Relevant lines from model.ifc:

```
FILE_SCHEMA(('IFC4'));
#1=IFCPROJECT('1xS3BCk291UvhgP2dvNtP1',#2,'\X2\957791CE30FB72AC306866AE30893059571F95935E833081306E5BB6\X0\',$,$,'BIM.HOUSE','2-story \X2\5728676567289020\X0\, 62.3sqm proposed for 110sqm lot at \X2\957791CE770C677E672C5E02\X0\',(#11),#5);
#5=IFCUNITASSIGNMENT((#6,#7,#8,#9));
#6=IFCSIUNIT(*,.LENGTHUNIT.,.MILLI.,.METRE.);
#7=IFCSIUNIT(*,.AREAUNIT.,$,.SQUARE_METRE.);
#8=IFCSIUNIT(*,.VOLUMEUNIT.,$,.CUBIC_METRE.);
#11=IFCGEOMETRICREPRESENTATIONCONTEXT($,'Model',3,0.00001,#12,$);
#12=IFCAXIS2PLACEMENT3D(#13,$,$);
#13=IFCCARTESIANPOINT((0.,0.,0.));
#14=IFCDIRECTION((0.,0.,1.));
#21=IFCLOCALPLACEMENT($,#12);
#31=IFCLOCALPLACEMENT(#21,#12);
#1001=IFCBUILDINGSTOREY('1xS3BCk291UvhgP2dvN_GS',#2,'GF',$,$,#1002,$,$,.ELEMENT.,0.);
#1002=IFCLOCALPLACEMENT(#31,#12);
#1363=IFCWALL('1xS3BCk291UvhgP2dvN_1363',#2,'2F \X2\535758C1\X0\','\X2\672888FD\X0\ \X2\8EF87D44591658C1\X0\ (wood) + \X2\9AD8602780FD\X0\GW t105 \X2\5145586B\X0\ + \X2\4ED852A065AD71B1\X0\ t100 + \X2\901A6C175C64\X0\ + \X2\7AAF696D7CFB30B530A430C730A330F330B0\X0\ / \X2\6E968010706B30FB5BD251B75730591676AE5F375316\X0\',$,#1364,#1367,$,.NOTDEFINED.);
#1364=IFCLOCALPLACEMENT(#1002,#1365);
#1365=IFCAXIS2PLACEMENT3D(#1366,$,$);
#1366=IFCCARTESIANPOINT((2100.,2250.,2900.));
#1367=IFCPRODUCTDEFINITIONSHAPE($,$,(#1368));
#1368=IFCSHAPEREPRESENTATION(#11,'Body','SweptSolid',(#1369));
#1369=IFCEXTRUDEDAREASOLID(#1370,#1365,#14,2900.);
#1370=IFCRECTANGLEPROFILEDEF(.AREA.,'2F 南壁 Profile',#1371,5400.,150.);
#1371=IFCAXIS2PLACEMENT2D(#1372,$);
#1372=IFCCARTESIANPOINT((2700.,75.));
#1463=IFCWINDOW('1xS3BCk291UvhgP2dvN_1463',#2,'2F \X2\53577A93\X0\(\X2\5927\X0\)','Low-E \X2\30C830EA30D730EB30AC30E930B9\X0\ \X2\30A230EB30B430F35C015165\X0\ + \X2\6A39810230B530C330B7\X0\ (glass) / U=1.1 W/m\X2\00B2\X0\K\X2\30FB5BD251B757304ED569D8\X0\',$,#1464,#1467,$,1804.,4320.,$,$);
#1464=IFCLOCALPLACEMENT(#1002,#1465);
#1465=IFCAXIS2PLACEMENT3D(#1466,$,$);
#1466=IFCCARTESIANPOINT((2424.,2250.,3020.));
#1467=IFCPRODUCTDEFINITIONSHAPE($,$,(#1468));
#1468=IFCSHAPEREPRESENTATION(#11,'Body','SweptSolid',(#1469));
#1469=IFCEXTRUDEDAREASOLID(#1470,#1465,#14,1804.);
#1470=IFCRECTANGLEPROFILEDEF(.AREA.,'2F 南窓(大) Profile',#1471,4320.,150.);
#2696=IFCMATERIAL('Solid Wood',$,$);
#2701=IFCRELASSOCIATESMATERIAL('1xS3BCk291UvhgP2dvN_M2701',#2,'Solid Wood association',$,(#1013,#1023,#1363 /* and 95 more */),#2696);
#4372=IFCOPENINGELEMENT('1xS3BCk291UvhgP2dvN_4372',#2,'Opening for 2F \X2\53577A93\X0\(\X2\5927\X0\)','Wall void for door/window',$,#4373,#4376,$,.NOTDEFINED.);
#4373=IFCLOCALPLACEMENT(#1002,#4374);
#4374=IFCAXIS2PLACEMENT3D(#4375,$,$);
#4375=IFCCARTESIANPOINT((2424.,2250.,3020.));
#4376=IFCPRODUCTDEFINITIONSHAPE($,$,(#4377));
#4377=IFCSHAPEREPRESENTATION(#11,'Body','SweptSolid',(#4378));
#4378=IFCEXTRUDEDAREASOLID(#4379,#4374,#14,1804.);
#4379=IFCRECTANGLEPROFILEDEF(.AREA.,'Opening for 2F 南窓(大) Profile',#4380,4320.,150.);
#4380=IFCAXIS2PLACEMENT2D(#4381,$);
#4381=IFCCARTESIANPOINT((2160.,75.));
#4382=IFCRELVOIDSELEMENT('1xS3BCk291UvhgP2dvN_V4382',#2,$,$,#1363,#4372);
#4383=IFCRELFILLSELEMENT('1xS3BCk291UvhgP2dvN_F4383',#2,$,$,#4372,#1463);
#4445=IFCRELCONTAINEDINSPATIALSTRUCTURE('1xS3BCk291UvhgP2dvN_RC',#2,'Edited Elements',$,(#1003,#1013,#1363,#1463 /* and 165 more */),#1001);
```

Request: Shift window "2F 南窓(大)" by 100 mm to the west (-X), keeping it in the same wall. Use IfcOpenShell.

```python
import ifcopenshell
import ifcopenshell.api.geometry
import ifcopenshell.util.placement
import ifcopenshell.util.unit

model = ifcopenshell.open("model.ifc")
unit_scale = ifcopenshell.util.unit.calculate_unit_scale(model)

window = model.by_id(1463)
opening = window.FillsVoids[0].RelatingOpeningElement
wall = opening.VoidsElements[0].RelatingBuildingElement

wall_matrix = ifcopenshell.util.placement.get_local_placement(wall.ObjectPlacement)
shift = wall_matrix[:3, 0] * -0.1 / unit_scale
before = ifcopenshell.util.placement.get_local_placement(window.ObjectPlacement)[:3, 3].copy()

# The window is not placed relative to its opening, so move both.
for product in (opening, window):
    matrix = ifcopenshell.util.placement.get_local_placement(product.ObjectPlacement)
    matrix[:3, 3] += shift
    ifcopenshell.api.geometry.edit_object_placement(model, product=product, matrix=matrix, is_si=False)

after = ifcopenshell.util.placement.get_local_placement(window.ObjectPlacement)[:3, 3]
print("window moved by", (after - before).round(3) + 0.0)

model.write("model_updated.ifc")
```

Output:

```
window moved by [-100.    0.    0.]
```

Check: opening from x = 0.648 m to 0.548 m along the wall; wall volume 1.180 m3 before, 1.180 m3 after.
